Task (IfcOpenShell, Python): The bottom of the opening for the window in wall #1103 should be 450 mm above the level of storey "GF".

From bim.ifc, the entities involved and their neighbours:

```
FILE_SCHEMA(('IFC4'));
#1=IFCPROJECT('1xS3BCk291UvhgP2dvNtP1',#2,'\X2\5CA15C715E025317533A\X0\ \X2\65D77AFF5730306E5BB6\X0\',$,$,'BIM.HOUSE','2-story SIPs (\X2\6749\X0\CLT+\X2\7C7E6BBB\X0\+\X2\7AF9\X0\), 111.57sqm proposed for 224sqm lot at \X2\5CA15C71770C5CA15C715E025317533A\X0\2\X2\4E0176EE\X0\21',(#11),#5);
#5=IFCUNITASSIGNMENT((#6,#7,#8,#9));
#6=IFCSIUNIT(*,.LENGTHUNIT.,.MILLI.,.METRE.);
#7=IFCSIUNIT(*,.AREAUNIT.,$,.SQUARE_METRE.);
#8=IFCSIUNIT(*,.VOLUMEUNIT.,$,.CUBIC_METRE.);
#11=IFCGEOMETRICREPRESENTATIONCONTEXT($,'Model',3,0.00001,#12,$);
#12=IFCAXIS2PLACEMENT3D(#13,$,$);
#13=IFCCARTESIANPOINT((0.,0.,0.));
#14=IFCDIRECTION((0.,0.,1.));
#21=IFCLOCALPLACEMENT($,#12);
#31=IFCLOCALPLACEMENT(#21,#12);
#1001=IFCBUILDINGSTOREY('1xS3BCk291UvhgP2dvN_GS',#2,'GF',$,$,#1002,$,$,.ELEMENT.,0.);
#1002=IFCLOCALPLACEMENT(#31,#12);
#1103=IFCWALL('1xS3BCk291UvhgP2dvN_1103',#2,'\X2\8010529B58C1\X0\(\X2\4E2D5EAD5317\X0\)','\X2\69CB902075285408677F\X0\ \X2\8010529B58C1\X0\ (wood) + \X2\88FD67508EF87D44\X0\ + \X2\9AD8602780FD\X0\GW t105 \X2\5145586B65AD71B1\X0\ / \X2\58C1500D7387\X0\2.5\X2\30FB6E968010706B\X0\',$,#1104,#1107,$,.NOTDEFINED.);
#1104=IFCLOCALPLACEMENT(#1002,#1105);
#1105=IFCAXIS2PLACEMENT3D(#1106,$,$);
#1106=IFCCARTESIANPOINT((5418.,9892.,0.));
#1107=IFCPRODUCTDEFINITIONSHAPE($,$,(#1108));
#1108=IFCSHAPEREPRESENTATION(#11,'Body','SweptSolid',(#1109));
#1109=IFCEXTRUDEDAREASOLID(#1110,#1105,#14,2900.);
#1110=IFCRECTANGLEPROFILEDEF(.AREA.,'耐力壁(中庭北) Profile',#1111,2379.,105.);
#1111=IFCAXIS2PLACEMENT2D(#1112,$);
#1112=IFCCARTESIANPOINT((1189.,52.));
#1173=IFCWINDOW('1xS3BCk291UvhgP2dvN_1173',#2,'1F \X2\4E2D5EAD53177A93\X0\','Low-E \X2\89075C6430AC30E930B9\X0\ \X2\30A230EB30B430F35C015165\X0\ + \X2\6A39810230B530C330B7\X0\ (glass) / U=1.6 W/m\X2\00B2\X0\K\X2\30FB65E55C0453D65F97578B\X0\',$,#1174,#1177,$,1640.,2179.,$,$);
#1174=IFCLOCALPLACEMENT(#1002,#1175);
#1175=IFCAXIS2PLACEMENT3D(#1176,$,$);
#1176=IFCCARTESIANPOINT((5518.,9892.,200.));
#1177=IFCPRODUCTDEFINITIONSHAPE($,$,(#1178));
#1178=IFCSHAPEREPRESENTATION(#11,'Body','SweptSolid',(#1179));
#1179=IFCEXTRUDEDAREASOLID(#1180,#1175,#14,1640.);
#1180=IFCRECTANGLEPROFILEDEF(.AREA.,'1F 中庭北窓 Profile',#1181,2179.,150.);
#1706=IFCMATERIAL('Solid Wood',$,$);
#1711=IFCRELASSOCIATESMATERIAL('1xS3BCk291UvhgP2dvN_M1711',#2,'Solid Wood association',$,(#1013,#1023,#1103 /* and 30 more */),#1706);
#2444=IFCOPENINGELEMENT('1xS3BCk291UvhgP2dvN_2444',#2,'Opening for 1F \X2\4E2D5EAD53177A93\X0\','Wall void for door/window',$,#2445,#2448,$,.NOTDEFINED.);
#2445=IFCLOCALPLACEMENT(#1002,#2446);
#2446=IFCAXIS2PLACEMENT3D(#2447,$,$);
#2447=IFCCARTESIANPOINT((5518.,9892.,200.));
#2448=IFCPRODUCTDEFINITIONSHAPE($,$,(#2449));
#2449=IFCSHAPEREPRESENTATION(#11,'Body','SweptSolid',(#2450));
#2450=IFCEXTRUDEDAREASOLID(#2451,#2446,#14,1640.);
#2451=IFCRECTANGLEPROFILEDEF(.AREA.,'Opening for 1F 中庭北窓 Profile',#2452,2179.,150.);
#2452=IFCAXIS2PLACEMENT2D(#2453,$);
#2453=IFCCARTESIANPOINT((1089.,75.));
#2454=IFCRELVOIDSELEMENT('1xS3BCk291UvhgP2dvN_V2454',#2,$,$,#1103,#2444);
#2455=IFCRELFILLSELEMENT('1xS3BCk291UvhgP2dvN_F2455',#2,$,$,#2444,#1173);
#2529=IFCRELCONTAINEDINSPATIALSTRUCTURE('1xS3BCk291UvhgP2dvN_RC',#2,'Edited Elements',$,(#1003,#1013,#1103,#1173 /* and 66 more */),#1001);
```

```python
import numpy as np
import ifcopenshell
import ifcopenshell.api.geometry
import ifcopenshell.geom
import ifcopenshell.util.element
import ifcopenshell.util.placement
import ifcopenshell.util.shape
import ifcopenshell.util.unit

model = ifcopenshell.open("bim.ifc")
unit_scale = ifcopenshell.util.unit.calculate_unit_scale(model)

window = model.by_guid("1xS3BCk291UvhgP2dvN_1173")
opening = window.FillsVoids[0].RelatingOpeningElement
storey = ifcopenshell.util.element.get_container(window, ifc_class="IfcBuildingStorey")
level = ifcopenshell.util.placement.get_local_placement(storey.ObjectPlacement)[2, 3]

# The opening's origin need not be at the sill, so measure its lowest point.
shape = ifcopenshell.geom.create_shape(ifcopenshell.geom.settings(), opening)
bottom = ifcopenshell.util.shape.get_shape_bottom_elevation(shape, shape.geometry) / unit_scale
dz = level + 450.0 - bottom

shift = np.array([0.0, 0.0, dz])
# The window is not placed relative to its opening, so move both.
for product in (opening, window):
    matrix = ifcopenshell.util.placement.get_local_placement(product.ObjectPlacement)
    matrix[:3, 3] += shift
    ifcopenshell.api.geometry.edit_object_placement(model, product=product, matrix=matrix, is_si=False)

print(f"moved by {dz * unit_scale:+.3f} m")

model.write("bim_updated.ifc")
```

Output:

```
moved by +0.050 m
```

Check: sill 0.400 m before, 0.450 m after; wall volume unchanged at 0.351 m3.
